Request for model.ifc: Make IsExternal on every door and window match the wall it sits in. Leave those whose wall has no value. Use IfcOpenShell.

First a look at what the model holds.

```python
import ifcopenshell
import ifcopenshell.util.element

model = ifcopenshell.open("model.ifc")
print(model.schema)
seen = {}
for e in model.by_type("IfcDoor") + model.by_type("IfcWindow"):
    if not e.FillsVoids:
        continue
    host = e.FillsVoids[0].RelatingOpeningElement.VoidsElements[0].RelatingBuildingElement
    own = ifcopenshell.util.element.get_pset(e, f"Pset_{e.is_a()[3:].removesuffix('StandardCase')}Common", "IsExternal")
    wall = ifcopenshell.util.element.get_pset(host, "Pset_WallCommon", "IsExternal")
    seen[e.is_a(), own, wall] = seen.get((e.is_a(), own, wall), 0) + 1
for (cls, own, wall), count in sorted(seen.items(), key=str):
    print(count, cls, "IsExternal:", own, "| host wall:", wall)
```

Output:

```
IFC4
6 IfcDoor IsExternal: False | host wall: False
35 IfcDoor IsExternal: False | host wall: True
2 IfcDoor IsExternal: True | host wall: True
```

```python
import ifcopenshell
import ifcopenshell.api.pset
import ifcopenshell.util.element

model = ifcopenshell.open("model.ifc")

count = 0
for ifc_class, pset_name in (("IfcDoor", "Pset_DoorCommon"), ("IfcWindow", "Pset_WindowCommon")):
    for e in model.by_type(ifc_class):
        if not e.FillsVoids:
            continue
        host = e.FillsVoids[0].RelatingOpeningElement.VoidsElements[0].RelatingBuildingElement
        external = ifcopenshell.util.element.get_pset(host, "Pset_WallCommon", "IsExternal")
        if external is None or ifcopenshell.util.element.get_pset(e, pset_name, "IsExternal") == external:
            continue
        pset = ifcopenshell.api.pset.add_pset(model, product=e, name=pset_name)
        ifcopenshell.api.pset.edit_pset(model, pset=pset, properties={"IsExternal": external})
        count += 1

print(count, "updated")

model.write("model_rev.ifc")
```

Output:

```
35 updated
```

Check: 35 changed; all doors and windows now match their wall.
